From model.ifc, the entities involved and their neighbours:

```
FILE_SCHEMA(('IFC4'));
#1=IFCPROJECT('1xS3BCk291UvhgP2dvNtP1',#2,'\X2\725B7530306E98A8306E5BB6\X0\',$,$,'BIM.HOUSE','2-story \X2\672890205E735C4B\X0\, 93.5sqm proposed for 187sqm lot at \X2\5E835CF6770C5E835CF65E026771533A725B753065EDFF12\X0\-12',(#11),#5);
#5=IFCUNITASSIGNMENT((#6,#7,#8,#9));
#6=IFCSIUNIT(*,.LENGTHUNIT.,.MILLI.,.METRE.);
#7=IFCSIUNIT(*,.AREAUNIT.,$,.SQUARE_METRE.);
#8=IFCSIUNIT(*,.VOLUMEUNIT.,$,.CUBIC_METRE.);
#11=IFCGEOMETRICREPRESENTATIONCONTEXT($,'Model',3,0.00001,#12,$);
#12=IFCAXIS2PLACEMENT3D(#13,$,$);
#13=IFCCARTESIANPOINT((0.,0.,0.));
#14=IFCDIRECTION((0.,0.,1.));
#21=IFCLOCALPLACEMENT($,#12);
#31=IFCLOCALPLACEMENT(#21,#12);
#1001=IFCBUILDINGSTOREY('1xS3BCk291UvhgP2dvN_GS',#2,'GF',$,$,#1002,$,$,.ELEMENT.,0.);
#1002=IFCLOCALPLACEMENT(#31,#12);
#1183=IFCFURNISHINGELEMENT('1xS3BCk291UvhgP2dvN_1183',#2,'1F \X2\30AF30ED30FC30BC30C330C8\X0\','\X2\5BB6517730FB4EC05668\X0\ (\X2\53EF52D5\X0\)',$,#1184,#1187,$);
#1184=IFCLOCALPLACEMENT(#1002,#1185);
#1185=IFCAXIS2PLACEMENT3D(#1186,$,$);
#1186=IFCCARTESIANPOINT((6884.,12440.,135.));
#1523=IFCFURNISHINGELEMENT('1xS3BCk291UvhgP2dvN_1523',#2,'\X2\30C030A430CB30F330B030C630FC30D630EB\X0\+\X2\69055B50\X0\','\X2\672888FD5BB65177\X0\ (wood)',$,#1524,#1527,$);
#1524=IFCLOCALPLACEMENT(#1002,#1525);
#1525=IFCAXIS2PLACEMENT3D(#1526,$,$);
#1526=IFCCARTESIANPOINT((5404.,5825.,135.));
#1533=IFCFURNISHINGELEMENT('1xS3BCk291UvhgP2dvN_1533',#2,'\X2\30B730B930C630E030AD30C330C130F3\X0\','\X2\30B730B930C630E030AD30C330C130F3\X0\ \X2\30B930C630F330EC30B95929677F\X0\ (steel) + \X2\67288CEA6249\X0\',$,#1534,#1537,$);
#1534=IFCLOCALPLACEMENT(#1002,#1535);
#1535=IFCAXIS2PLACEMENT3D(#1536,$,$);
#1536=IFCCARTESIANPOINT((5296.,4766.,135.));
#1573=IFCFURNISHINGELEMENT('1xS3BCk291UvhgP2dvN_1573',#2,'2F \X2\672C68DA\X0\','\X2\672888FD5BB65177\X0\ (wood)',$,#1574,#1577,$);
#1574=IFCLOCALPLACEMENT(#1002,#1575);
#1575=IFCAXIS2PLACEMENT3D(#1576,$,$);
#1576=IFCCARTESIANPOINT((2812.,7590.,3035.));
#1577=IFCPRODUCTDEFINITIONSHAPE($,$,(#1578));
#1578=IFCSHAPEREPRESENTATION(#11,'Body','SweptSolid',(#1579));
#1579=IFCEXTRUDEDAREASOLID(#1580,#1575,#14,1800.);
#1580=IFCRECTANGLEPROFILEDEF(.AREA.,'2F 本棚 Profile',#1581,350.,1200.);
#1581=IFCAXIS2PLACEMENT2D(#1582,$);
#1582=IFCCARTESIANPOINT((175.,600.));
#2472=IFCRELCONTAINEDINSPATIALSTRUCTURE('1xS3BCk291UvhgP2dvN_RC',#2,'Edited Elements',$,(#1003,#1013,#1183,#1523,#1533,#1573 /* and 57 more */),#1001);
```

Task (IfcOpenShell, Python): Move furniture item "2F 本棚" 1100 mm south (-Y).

```python
import ifcopenshell
import ifcopenshell.api.geometry
import ifcopenshell.util.placement

model = ifcopenshell.open("model.ifc")

item = model.by_guid("1xS3BCk291UvhgP2dvN_1573")
matrix = ifcopenshell.util.placement.get_local_placement(item.ObjectPlacement)
matrix[1, 3] -= 1100.0
ifcopenshell.api.geometry.edit_object_placement(model, product=item, matrix=matrix, is_si=False)

print(ifcopenshell.util.placement.get_local_placement(item.ObjectPlacement).round(3) + 0.0)

model.write("model_edited.ifc")
```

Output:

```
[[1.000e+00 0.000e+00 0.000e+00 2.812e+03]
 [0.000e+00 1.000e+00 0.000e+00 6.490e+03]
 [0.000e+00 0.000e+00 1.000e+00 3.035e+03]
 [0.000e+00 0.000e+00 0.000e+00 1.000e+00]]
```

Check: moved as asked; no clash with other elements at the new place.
